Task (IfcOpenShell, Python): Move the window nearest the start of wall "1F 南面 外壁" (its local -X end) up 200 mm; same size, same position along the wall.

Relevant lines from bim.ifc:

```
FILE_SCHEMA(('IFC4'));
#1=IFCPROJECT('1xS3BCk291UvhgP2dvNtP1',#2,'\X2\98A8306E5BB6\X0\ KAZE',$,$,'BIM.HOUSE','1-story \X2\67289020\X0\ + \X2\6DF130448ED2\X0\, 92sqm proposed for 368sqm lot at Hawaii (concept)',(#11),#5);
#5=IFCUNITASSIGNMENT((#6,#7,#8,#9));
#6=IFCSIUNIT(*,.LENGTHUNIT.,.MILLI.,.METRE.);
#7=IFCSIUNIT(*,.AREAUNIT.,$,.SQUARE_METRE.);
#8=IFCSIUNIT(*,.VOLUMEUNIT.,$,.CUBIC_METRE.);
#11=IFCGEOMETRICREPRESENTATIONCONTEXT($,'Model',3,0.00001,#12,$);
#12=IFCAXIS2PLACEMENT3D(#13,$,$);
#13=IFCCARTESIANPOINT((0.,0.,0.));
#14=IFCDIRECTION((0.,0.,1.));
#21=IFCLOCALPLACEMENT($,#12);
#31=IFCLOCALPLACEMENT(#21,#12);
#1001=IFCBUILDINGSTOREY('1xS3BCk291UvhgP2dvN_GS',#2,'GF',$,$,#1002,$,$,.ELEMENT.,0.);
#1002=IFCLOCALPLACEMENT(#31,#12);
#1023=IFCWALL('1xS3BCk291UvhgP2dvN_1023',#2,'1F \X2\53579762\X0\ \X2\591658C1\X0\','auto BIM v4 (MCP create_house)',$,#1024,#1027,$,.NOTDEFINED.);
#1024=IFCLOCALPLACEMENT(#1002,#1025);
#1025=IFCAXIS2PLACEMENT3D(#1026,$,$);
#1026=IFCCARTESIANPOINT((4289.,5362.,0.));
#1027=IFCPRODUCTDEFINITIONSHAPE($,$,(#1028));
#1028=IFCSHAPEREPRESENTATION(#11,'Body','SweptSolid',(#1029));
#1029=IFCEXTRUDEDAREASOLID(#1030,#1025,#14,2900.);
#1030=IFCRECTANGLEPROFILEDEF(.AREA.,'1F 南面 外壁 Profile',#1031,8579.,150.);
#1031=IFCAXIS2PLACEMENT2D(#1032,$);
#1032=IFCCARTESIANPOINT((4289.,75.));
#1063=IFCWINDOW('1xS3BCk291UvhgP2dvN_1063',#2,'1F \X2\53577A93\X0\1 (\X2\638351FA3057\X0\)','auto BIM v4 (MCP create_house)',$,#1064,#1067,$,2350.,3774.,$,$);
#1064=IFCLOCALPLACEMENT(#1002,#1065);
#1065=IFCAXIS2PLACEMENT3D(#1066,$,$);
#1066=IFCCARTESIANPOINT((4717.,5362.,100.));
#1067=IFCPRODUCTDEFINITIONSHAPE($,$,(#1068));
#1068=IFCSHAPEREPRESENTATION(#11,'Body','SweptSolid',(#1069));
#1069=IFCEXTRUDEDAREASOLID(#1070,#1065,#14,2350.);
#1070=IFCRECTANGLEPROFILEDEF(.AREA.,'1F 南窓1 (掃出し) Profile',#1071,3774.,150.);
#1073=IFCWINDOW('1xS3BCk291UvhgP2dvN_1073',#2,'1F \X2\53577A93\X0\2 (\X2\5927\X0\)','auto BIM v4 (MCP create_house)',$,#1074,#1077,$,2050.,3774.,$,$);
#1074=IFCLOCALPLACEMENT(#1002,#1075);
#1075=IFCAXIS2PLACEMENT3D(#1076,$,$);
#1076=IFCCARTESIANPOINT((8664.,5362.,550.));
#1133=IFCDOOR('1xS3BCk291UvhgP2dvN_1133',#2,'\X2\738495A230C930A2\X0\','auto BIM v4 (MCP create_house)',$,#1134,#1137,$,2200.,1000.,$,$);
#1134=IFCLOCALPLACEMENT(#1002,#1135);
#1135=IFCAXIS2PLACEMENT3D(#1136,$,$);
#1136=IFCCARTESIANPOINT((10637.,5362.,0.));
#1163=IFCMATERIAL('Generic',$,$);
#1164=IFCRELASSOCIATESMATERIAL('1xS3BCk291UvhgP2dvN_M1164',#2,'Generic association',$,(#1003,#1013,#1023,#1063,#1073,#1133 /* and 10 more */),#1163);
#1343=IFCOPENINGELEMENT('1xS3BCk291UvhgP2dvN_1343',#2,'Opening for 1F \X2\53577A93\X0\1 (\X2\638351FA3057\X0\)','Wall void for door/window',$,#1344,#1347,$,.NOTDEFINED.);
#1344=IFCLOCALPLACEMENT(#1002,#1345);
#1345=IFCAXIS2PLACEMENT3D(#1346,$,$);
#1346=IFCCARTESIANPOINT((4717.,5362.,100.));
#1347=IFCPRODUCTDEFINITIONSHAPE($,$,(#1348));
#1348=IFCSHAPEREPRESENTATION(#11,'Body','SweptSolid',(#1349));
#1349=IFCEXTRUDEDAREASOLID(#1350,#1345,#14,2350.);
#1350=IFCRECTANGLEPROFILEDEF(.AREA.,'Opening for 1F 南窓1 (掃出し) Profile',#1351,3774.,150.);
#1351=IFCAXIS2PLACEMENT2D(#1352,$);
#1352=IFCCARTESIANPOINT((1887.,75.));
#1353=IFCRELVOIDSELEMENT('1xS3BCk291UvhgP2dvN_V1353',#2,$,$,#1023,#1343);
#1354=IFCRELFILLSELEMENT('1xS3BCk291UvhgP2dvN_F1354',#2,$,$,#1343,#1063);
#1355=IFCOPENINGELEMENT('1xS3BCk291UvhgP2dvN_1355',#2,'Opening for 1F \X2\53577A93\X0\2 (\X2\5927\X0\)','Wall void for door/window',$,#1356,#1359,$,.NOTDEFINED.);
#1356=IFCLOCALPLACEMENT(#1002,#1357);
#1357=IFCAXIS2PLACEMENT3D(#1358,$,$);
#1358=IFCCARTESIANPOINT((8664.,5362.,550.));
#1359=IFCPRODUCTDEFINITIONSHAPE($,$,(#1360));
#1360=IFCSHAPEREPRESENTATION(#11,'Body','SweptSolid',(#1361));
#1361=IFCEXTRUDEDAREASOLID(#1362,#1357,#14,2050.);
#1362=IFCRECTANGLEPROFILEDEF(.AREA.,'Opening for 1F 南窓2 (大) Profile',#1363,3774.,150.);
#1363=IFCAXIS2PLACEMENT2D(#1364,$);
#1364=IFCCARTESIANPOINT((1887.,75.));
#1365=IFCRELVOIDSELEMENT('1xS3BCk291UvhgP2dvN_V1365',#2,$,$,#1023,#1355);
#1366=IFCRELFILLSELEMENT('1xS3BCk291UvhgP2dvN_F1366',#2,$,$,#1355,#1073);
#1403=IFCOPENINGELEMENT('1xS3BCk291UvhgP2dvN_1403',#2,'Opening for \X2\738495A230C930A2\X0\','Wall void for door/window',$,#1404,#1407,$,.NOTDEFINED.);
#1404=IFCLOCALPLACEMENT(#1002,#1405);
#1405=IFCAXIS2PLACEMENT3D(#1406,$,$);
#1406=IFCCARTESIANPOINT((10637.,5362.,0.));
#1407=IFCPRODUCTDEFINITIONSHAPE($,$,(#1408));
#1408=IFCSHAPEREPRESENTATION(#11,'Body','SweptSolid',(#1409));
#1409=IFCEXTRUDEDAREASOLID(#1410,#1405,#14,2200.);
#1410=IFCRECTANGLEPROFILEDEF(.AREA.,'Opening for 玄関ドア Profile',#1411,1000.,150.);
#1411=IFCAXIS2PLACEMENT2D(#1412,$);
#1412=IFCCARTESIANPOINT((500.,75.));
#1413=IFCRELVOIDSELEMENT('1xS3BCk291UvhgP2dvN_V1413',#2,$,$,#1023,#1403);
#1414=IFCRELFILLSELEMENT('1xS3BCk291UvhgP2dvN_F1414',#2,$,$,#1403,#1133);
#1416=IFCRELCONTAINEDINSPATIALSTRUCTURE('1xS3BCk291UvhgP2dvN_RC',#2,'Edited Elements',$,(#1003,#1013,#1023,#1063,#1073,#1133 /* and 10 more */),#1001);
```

```python
import numpy as np
import ifcopenshell
import ifcopenshell.api.geometry
import ifcopenshell.util.placement
import ifcopenshell.util.unit

model = ifcopenshell.open("bim.ifc")
unit_scale = ifcopenshell.util.unit.calculate_unit_scale(model)

window = model.by_guid("1xS3BCk291UvhgP2dvN_1063")
opening = window.FillsVoids[0].RelatingOpeningElement
dz = 0.2 / unit_scale

shift = np.array([0.0, 0.0, dz])
# The window is not placed relative to its opening, so move both.
for product in (opening, window):
    matrix = ifcopenshell.util.placement.get_local_placement(product.ObjectPlacement)
    matrix[:3, 3] += shift
    ifcopenshell.api.geometry.edit_object_placement(model, product=product, matrix=matrix, is_si=False)

print(f"moved by {dz * unit_scale:+.3f} m")

model.write("bim-out.ifc")
```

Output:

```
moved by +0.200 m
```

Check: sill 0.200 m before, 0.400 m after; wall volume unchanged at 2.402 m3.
